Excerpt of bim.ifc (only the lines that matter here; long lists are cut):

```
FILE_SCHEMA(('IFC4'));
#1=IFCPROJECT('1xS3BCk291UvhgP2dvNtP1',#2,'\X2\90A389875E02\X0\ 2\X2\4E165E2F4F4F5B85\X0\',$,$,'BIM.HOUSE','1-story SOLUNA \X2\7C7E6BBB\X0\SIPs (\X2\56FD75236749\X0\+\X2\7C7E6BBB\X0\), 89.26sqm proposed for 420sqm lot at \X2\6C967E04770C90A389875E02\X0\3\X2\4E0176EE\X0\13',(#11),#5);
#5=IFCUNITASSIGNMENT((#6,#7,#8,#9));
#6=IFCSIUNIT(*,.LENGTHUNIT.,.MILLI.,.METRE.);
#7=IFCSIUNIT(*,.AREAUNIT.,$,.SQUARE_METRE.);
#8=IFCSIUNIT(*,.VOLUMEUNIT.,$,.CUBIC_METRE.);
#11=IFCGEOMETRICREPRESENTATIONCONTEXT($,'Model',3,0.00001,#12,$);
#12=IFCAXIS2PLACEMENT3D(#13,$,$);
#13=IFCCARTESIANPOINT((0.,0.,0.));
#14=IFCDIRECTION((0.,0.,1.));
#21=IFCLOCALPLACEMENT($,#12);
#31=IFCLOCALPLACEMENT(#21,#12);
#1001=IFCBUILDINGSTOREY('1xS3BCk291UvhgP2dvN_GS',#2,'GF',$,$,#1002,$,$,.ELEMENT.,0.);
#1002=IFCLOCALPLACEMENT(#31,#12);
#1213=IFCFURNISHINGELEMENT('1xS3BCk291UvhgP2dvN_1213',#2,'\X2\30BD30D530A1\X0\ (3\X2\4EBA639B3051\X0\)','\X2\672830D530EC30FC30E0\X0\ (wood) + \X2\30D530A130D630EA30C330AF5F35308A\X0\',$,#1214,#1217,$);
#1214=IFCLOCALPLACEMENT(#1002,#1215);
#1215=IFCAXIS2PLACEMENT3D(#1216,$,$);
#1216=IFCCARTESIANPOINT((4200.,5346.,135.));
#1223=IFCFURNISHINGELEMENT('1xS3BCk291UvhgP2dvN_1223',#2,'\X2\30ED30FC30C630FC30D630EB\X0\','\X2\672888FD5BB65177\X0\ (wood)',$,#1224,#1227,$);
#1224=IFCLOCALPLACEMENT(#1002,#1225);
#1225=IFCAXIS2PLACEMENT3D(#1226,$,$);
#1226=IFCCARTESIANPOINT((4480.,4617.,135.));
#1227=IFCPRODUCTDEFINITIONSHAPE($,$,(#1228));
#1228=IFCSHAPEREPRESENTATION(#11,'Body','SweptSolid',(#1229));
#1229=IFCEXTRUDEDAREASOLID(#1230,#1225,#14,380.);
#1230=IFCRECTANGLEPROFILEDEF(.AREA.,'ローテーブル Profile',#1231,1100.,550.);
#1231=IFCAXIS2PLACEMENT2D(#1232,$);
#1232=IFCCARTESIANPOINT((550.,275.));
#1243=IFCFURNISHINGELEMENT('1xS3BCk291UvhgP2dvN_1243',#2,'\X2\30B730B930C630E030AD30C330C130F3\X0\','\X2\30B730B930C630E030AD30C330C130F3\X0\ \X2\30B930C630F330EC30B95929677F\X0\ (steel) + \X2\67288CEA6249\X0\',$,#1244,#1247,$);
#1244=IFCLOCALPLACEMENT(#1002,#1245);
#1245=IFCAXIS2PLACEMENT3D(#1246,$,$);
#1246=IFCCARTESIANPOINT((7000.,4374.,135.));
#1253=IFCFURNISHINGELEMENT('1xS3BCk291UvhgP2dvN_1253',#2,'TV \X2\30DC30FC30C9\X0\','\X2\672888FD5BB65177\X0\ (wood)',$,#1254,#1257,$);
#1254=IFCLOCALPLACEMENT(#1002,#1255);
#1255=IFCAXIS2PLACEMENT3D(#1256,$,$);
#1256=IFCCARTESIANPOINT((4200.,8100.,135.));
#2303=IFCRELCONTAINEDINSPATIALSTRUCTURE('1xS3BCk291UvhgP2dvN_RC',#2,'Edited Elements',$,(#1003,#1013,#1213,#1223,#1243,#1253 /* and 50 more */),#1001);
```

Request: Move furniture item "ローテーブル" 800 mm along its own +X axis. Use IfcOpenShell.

```python
import ifcopenshell
import ifcopenshell.api.geometry
import ifcopenshell.util.placement
import ifcopenshell.util.unit

model = ifcopenshell.open("bim.ifc")
unit_scale = ifcopenshell.util.unit.calculate_unit_scale(model)

item = model.by_guid("1xS3BCk291UvhgP2dvN_1223")
matrix = ifcopenshell.util.placement.get_local_placement(item.ObjectPlacement)
matrix[:3, 3] += matrix[:3, 0] * 0.8 / unit_scale
ifcopenshell.api.geometry.edit_object_placement(model, product=item, matrix=matrix, is_si=False)

print(ifcopenshell.util.placement.get_local_placement(item.ObjectPlacement).round(3) + 0.0)

model.write("bim_rev.ifc")
```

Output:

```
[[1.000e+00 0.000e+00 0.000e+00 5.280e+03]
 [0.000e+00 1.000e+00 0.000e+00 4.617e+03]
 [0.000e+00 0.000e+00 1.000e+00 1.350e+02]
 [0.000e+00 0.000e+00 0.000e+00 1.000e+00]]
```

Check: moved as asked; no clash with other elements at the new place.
